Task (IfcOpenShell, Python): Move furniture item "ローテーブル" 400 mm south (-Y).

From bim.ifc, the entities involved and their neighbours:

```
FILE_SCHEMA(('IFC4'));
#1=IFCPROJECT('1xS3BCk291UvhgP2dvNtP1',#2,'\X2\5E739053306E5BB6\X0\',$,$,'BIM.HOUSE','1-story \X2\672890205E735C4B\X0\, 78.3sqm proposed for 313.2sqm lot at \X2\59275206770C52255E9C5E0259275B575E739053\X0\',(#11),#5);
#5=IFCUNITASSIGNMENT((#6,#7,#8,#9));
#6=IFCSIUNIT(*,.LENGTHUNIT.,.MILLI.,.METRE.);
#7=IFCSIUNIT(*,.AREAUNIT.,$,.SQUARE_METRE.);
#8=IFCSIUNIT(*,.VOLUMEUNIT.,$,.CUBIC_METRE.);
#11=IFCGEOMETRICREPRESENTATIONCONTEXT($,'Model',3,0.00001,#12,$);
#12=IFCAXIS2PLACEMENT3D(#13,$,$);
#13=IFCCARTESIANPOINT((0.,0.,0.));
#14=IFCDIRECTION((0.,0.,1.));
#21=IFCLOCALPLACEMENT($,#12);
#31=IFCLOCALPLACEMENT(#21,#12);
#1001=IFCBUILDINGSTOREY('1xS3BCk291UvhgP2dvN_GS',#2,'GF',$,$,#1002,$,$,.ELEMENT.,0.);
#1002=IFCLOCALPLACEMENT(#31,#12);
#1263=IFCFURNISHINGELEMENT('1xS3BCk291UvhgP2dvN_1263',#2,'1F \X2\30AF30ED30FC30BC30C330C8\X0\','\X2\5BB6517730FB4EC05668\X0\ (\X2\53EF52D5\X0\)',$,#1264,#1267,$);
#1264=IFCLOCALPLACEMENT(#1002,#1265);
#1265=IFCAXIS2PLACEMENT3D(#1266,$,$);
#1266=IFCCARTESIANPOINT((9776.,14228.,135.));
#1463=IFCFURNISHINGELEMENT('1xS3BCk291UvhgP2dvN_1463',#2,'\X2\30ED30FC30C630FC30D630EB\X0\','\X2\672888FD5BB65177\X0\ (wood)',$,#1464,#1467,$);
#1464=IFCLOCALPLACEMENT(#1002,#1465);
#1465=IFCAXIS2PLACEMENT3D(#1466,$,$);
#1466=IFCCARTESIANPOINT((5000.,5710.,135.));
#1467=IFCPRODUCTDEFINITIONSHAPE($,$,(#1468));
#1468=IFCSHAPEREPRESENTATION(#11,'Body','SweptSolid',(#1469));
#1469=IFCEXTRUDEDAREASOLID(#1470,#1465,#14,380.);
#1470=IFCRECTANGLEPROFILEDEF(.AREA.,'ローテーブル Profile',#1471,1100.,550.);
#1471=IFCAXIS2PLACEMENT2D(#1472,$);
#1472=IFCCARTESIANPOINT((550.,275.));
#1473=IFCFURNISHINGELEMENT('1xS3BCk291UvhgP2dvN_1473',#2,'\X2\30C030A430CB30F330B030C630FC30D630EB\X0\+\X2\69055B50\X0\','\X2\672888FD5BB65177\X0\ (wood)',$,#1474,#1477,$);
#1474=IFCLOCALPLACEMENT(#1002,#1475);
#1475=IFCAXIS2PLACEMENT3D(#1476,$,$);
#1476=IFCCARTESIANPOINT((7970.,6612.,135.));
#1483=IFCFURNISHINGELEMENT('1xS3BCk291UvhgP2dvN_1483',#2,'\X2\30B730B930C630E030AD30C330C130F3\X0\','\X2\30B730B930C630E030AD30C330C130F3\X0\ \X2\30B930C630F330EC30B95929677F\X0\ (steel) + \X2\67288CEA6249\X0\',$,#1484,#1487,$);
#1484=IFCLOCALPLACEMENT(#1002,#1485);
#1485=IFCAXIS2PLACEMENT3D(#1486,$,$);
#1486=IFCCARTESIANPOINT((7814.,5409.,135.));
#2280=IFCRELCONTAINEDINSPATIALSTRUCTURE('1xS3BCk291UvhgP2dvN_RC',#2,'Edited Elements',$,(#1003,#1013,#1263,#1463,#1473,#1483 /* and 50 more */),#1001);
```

```python
import ifcopenshell
import ifcopenshell.api.geometry
import ifcopenshell.util.placement
import ifcopenshell.util.unit

model = ifcopenshell.open("bim.ifc")
unit_scale = ifcopenshell.util.unit.calculate_unit_scale(model)

item = model.by_guid("1xS3BCk291UvhgP2dvN_1463")
matrix = ifcopenshell.util.placement.get_local_placement(item.ObjectPlacement)
matrix[1, 3] -= 0.4 / unit_scale
ifcopenshell.api.geometry.edit_object_placement(model, product=item, matrix=matrix, is_si=False)

print(ifcopenshell.util.placement.get_local_placement(item.ObjectPlacement).round(3) + 0.0)

model.write("bim_edited.ifc")
```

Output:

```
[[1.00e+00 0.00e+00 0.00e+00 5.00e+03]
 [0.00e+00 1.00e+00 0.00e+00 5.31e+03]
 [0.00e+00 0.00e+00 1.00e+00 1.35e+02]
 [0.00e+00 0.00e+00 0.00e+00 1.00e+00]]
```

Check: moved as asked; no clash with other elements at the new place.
